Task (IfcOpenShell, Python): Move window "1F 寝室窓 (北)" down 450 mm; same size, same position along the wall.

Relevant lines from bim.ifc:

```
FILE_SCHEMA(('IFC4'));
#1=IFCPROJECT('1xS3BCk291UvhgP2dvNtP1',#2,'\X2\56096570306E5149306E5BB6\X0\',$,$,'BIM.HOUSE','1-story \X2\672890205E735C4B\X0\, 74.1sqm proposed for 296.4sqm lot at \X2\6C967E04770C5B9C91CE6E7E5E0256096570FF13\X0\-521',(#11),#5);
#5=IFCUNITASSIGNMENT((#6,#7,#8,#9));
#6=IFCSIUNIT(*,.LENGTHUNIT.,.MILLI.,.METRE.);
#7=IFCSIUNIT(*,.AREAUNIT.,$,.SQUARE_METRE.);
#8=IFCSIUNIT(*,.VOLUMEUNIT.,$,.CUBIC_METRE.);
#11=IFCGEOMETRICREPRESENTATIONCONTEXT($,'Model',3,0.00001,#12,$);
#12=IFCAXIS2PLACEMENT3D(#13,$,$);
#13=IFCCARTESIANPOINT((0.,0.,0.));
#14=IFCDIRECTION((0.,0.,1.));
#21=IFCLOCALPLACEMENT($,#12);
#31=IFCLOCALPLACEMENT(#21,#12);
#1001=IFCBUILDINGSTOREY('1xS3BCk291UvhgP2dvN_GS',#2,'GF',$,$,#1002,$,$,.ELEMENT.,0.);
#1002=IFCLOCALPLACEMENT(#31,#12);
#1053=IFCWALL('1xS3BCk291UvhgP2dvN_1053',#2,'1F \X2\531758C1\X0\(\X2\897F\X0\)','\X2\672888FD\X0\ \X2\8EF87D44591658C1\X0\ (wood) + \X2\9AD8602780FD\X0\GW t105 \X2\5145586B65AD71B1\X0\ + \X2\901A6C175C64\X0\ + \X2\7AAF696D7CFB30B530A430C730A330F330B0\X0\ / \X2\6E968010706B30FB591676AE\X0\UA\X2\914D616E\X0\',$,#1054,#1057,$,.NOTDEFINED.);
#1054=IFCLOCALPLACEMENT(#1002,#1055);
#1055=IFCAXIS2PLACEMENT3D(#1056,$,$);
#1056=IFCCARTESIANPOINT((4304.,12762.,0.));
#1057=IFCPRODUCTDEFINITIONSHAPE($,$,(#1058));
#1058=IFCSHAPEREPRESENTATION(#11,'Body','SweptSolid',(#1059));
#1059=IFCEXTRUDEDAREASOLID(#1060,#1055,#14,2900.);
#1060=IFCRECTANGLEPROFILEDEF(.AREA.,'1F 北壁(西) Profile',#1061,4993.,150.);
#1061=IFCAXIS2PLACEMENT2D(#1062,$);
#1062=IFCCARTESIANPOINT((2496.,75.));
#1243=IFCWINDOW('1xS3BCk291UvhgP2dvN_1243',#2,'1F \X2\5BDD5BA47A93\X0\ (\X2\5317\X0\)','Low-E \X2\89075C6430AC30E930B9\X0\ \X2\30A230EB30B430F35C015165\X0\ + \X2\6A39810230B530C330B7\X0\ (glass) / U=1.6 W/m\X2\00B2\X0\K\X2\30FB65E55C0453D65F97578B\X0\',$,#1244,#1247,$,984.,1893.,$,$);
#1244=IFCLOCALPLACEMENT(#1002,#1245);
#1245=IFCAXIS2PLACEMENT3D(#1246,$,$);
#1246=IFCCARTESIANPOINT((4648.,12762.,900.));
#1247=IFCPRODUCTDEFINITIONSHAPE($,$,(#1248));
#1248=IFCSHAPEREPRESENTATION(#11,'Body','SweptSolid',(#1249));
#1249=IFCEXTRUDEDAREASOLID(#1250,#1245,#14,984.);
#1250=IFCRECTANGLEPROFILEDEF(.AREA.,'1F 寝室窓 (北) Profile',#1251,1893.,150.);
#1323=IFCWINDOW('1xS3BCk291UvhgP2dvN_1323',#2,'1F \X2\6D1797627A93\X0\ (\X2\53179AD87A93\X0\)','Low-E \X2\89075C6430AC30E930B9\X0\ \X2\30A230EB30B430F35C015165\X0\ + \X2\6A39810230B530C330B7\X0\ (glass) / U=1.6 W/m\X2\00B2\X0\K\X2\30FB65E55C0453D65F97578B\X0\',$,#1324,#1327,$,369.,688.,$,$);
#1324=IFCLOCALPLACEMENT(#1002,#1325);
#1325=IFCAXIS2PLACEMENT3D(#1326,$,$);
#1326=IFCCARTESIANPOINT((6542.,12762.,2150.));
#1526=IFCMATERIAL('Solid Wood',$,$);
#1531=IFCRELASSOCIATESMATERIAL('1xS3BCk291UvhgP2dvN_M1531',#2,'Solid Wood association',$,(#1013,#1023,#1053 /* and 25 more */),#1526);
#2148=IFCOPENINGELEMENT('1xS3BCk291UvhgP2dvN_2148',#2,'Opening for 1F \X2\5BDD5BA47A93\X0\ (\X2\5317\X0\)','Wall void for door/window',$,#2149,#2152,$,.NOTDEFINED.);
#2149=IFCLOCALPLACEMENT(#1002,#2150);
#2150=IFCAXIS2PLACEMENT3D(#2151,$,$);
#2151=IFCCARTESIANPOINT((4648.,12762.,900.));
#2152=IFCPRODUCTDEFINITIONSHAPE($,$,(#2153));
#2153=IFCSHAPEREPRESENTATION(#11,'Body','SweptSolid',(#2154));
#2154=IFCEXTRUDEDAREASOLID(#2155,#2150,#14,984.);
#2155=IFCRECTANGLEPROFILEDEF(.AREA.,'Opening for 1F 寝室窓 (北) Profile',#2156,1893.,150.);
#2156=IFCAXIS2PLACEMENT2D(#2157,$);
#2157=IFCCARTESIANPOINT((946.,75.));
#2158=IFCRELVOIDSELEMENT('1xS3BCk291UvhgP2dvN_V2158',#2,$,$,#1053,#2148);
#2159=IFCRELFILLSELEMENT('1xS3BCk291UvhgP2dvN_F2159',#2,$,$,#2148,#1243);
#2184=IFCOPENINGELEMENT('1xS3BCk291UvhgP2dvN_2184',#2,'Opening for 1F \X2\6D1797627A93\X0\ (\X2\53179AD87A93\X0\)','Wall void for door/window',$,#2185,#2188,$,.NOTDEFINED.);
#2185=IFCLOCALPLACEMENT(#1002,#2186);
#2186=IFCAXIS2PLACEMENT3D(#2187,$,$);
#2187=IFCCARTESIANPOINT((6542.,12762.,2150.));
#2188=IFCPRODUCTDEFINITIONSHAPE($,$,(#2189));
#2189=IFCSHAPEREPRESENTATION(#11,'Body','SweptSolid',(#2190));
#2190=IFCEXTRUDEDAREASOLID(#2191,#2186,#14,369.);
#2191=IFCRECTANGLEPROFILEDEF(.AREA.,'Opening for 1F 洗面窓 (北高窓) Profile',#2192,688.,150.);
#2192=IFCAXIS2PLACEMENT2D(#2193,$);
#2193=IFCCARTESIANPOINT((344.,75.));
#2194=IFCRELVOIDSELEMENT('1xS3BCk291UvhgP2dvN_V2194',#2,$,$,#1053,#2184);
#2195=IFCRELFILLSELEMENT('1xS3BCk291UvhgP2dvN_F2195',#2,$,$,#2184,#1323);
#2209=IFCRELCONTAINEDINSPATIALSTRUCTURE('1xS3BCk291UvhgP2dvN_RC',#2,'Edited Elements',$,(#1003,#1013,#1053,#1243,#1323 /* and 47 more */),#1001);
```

```python
import numpy as np
import ifcopenshell
import ifcopenshell.api.geometry
import ifcopenshell.util.placement
import ifcopenshell.util.unit

model = ifcopenshell.open("bim.ifc")
unit_scale = ifcopenshell.util.unit.calculate_unit_scale(model)

window = model.by_guid("1xS3BCk291UvhgP2dvN_1243")
opening = window.FillsVoids[0].RelatingOpeningElement
dz = -0.45 / unit_scale

shift = np.array([0.0, 0.0, dz])
# The window is not placed relative to its opening, so move both.
for product in (opening, window):
    matrix = ifcopenshell.util.placement.get_local_placement(product.ObjectPlacement)
    matrix[:3, 3] += shift
    ifcopenshell.api.geometry.edit_object_placement(model, product=product, matrix=matrix, is_si=False)

print(f"moved by {dz * unit_scale:+.3f} m")

model.write("bim_v2.ifc")
```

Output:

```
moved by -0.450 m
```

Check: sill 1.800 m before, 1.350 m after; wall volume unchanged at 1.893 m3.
